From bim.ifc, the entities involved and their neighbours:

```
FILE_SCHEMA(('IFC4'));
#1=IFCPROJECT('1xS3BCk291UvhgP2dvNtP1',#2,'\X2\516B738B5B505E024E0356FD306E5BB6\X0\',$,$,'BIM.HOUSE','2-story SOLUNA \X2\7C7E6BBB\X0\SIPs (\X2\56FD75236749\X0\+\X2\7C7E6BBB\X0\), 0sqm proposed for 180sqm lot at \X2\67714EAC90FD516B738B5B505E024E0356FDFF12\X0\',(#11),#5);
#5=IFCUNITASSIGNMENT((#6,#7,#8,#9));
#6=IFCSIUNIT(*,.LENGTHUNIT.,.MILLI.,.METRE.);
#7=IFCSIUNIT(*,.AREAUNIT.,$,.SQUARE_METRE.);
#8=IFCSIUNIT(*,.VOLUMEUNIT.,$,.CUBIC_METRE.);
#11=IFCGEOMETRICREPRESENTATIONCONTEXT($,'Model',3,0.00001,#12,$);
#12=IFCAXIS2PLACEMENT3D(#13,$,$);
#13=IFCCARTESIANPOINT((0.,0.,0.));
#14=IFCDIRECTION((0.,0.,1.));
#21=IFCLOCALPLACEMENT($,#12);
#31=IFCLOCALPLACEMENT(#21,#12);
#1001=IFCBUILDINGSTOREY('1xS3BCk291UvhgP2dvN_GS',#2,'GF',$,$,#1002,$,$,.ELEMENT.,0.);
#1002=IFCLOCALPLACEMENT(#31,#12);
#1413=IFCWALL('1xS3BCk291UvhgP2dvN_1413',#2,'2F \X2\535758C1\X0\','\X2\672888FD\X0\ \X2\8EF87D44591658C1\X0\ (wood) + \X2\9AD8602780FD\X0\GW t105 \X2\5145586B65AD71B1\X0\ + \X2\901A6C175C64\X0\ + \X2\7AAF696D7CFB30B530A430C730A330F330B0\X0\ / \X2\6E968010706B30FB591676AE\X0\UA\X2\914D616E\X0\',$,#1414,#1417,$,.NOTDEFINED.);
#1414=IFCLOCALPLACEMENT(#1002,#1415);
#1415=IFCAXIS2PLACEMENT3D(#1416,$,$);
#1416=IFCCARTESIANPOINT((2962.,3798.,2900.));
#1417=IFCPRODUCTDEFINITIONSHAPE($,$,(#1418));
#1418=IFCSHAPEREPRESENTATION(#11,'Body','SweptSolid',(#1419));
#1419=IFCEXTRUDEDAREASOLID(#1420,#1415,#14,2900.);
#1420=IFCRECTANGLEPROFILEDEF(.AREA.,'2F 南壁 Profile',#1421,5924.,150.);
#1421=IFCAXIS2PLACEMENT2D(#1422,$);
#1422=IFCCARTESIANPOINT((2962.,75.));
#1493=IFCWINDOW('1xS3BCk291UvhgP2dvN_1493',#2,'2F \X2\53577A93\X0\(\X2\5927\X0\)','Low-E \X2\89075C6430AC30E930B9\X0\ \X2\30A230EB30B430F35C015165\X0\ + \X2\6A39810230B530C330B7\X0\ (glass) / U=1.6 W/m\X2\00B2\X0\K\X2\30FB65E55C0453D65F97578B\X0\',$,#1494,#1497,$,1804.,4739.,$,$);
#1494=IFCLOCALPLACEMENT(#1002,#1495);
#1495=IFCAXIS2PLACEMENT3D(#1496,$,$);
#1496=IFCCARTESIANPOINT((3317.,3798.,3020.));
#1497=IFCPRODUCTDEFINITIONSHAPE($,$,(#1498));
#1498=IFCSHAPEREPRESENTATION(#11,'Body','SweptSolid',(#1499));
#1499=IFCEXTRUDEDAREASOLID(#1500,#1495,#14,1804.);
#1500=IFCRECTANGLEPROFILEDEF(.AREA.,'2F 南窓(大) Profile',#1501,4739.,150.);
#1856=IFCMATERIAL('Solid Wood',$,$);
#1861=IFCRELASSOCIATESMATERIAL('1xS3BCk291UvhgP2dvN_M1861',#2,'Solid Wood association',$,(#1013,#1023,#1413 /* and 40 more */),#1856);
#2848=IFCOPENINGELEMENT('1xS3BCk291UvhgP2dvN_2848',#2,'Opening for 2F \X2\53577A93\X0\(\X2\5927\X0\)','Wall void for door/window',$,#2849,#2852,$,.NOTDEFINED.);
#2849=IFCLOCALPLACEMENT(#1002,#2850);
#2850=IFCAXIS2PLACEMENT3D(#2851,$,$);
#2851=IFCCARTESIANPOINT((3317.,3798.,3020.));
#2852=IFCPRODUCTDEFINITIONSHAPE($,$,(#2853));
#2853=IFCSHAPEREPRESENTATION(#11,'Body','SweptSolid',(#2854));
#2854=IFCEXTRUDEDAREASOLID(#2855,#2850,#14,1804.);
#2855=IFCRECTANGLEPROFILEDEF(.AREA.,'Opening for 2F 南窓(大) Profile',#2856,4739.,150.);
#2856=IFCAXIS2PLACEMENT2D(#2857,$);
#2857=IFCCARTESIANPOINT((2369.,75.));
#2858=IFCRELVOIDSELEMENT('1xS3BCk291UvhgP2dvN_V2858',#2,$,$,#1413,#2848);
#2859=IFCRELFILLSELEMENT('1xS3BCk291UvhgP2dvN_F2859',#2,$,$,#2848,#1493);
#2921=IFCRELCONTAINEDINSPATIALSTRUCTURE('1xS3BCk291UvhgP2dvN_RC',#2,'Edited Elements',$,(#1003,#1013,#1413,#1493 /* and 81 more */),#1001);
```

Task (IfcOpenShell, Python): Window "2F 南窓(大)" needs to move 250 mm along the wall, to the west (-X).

```python
import ifcopenshell
import ifcopenshell.api.geometry
import ifcopenshell.util.placement
import ifcopenshell.util.unit

model = ifcopenshell.open("bim.ifc")
unit_scale = ifcopenshell.util.unit.calculate_unit_scale(model)

window = model.by_guid("1xS3BCk291UvhgP2dvN_1493")
opening = window.FillsVoids[0].RelatingOpeningElement
wall = opening.VoidsElements[0].RelatingBuildingElement

wall_matrix = ifcopenshell.util.placement.get_local_placement(wall.ObjectPlacement)
shift = wall_matrix[:3, 0] * -0.25 / unit_scale
before = ifcopenshell.util.placement.get_local_placement(window.ObjectPlacement)[:3, 3].copy()

# The window is not placed relative to its opening, so move both.
for product in (opening, window):
    matrix = ifcopenshell.util.placement.get_local_placement(product.ObjectPlacement)
    matrix[:3, 3] += shift
    ifcopenshell.api.geometry.edit_object_placement(model, product=product, matrix=matrix, is_si=False)

after = ifcopenshell.util.placement.get_local_placement(window.ObjectPlacement)[:3, 3]
print("window moved by", (after - before).round(3) + 0.0)

model.write("bim_rev.ifc")
```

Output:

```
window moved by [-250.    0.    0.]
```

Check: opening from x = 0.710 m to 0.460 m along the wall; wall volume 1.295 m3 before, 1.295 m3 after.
